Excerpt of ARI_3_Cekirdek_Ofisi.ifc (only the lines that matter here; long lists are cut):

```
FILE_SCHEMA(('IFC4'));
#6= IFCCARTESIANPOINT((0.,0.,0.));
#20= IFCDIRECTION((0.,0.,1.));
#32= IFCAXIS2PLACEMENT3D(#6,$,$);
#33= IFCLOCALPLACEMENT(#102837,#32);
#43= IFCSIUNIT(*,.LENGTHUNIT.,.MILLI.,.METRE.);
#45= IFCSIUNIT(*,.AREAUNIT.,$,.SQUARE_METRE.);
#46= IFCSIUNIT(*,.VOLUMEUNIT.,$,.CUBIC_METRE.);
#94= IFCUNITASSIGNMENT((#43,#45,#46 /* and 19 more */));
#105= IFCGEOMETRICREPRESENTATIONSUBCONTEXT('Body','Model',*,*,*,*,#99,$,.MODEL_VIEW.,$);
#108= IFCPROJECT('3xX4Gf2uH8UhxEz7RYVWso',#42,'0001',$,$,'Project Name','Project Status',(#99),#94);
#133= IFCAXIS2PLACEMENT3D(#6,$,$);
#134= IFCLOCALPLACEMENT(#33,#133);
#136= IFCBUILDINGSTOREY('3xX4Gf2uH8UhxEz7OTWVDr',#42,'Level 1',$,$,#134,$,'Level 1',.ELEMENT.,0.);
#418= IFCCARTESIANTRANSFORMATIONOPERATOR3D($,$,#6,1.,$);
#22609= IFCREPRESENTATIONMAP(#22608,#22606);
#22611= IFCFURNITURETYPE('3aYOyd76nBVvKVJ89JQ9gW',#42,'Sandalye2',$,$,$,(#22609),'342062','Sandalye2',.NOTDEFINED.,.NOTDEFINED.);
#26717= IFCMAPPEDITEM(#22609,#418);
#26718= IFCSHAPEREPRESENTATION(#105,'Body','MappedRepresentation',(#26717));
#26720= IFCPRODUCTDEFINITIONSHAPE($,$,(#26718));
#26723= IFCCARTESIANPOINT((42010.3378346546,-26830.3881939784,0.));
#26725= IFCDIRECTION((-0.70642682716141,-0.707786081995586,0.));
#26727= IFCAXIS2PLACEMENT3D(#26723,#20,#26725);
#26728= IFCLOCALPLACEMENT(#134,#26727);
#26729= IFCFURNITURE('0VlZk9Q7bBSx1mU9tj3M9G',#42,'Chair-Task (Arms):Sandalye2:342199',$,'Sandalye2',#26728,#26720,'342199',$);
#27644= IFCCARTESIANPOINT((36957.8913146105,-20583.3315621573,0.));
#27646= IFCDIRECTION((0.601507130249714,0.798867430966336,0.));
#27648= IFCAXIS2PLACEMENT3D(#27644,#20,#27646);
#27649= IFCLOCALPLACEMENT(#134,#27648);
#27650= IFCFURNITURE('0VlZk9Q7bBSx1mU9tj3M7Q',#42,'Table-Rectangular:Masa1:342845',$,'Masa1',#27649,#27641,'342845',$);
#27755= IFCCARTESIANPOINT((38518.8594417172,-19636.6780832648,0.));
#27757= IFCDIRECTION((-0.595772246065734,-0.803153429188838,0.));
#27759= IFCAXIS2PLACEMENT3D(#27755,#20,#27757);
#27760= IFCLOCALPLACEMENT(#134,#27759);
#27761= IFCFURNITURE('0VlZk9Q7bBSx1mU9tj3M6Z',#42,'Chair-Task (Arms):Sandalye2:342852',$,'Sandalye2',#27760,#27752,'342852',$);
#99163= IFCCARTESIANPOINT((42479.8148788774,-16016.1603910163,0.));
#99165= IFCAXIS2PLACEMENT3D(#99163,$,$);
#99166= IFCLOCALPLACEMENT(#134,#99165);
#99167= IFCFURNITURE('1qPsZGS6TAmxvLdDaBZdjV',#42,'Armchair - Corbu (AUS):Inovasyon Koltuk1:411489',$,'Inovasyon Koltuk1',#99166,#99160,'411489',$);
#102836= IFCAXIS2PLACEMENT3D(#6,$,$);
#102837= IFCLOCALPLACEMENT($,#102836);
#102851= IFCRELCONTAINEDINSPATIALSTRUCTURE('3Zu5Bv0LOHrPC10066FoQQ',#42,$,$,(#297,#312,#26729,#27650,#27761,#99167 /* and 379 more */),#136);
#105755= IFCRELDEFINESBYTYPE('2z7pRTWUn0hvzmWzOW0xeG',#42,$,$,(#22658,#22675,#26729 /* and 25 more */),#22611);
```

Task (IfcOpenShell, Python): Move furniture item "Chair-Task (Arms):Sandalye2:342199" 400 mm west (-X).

```python
import ifcopenshell
import ifcopenshell.api.geometry
import ifcopenshell.util.placement
import ifcopenshell.util.unit

model = ifcopenshell.open("ARI_3_Cekirdek_Ofisi.ifc")
unit_scale = ifcopenshell.util.unit.calculate_unit_scale(model)

item = model.by_id(26729)
matrix = ifcopenshell.util.placement.get_local_placement(item.ObjectPlacement)
matrix[0, 3] -= 0.4 / unit_scale
ifcopenshell.api.geometry.edit_object_placement(model, product=item, matrix=matrix, is_si=False)

print(ifcopenshell.util.placement.get_local_placement(item.ObjectPlacement).round(3) + 0.0)

model.write("ARI_3_Cekirdek_Ofisi_v2.ifc")
```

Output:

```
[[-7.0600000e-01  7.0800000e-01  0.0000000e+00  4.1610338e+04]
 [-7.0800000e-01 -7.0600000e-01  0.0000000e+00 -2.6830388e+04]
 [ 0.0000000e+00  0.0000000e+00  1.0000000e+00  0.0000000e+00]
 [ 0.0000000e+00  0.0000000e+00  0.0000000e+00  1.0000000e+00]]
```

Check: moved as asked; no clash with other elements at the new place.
